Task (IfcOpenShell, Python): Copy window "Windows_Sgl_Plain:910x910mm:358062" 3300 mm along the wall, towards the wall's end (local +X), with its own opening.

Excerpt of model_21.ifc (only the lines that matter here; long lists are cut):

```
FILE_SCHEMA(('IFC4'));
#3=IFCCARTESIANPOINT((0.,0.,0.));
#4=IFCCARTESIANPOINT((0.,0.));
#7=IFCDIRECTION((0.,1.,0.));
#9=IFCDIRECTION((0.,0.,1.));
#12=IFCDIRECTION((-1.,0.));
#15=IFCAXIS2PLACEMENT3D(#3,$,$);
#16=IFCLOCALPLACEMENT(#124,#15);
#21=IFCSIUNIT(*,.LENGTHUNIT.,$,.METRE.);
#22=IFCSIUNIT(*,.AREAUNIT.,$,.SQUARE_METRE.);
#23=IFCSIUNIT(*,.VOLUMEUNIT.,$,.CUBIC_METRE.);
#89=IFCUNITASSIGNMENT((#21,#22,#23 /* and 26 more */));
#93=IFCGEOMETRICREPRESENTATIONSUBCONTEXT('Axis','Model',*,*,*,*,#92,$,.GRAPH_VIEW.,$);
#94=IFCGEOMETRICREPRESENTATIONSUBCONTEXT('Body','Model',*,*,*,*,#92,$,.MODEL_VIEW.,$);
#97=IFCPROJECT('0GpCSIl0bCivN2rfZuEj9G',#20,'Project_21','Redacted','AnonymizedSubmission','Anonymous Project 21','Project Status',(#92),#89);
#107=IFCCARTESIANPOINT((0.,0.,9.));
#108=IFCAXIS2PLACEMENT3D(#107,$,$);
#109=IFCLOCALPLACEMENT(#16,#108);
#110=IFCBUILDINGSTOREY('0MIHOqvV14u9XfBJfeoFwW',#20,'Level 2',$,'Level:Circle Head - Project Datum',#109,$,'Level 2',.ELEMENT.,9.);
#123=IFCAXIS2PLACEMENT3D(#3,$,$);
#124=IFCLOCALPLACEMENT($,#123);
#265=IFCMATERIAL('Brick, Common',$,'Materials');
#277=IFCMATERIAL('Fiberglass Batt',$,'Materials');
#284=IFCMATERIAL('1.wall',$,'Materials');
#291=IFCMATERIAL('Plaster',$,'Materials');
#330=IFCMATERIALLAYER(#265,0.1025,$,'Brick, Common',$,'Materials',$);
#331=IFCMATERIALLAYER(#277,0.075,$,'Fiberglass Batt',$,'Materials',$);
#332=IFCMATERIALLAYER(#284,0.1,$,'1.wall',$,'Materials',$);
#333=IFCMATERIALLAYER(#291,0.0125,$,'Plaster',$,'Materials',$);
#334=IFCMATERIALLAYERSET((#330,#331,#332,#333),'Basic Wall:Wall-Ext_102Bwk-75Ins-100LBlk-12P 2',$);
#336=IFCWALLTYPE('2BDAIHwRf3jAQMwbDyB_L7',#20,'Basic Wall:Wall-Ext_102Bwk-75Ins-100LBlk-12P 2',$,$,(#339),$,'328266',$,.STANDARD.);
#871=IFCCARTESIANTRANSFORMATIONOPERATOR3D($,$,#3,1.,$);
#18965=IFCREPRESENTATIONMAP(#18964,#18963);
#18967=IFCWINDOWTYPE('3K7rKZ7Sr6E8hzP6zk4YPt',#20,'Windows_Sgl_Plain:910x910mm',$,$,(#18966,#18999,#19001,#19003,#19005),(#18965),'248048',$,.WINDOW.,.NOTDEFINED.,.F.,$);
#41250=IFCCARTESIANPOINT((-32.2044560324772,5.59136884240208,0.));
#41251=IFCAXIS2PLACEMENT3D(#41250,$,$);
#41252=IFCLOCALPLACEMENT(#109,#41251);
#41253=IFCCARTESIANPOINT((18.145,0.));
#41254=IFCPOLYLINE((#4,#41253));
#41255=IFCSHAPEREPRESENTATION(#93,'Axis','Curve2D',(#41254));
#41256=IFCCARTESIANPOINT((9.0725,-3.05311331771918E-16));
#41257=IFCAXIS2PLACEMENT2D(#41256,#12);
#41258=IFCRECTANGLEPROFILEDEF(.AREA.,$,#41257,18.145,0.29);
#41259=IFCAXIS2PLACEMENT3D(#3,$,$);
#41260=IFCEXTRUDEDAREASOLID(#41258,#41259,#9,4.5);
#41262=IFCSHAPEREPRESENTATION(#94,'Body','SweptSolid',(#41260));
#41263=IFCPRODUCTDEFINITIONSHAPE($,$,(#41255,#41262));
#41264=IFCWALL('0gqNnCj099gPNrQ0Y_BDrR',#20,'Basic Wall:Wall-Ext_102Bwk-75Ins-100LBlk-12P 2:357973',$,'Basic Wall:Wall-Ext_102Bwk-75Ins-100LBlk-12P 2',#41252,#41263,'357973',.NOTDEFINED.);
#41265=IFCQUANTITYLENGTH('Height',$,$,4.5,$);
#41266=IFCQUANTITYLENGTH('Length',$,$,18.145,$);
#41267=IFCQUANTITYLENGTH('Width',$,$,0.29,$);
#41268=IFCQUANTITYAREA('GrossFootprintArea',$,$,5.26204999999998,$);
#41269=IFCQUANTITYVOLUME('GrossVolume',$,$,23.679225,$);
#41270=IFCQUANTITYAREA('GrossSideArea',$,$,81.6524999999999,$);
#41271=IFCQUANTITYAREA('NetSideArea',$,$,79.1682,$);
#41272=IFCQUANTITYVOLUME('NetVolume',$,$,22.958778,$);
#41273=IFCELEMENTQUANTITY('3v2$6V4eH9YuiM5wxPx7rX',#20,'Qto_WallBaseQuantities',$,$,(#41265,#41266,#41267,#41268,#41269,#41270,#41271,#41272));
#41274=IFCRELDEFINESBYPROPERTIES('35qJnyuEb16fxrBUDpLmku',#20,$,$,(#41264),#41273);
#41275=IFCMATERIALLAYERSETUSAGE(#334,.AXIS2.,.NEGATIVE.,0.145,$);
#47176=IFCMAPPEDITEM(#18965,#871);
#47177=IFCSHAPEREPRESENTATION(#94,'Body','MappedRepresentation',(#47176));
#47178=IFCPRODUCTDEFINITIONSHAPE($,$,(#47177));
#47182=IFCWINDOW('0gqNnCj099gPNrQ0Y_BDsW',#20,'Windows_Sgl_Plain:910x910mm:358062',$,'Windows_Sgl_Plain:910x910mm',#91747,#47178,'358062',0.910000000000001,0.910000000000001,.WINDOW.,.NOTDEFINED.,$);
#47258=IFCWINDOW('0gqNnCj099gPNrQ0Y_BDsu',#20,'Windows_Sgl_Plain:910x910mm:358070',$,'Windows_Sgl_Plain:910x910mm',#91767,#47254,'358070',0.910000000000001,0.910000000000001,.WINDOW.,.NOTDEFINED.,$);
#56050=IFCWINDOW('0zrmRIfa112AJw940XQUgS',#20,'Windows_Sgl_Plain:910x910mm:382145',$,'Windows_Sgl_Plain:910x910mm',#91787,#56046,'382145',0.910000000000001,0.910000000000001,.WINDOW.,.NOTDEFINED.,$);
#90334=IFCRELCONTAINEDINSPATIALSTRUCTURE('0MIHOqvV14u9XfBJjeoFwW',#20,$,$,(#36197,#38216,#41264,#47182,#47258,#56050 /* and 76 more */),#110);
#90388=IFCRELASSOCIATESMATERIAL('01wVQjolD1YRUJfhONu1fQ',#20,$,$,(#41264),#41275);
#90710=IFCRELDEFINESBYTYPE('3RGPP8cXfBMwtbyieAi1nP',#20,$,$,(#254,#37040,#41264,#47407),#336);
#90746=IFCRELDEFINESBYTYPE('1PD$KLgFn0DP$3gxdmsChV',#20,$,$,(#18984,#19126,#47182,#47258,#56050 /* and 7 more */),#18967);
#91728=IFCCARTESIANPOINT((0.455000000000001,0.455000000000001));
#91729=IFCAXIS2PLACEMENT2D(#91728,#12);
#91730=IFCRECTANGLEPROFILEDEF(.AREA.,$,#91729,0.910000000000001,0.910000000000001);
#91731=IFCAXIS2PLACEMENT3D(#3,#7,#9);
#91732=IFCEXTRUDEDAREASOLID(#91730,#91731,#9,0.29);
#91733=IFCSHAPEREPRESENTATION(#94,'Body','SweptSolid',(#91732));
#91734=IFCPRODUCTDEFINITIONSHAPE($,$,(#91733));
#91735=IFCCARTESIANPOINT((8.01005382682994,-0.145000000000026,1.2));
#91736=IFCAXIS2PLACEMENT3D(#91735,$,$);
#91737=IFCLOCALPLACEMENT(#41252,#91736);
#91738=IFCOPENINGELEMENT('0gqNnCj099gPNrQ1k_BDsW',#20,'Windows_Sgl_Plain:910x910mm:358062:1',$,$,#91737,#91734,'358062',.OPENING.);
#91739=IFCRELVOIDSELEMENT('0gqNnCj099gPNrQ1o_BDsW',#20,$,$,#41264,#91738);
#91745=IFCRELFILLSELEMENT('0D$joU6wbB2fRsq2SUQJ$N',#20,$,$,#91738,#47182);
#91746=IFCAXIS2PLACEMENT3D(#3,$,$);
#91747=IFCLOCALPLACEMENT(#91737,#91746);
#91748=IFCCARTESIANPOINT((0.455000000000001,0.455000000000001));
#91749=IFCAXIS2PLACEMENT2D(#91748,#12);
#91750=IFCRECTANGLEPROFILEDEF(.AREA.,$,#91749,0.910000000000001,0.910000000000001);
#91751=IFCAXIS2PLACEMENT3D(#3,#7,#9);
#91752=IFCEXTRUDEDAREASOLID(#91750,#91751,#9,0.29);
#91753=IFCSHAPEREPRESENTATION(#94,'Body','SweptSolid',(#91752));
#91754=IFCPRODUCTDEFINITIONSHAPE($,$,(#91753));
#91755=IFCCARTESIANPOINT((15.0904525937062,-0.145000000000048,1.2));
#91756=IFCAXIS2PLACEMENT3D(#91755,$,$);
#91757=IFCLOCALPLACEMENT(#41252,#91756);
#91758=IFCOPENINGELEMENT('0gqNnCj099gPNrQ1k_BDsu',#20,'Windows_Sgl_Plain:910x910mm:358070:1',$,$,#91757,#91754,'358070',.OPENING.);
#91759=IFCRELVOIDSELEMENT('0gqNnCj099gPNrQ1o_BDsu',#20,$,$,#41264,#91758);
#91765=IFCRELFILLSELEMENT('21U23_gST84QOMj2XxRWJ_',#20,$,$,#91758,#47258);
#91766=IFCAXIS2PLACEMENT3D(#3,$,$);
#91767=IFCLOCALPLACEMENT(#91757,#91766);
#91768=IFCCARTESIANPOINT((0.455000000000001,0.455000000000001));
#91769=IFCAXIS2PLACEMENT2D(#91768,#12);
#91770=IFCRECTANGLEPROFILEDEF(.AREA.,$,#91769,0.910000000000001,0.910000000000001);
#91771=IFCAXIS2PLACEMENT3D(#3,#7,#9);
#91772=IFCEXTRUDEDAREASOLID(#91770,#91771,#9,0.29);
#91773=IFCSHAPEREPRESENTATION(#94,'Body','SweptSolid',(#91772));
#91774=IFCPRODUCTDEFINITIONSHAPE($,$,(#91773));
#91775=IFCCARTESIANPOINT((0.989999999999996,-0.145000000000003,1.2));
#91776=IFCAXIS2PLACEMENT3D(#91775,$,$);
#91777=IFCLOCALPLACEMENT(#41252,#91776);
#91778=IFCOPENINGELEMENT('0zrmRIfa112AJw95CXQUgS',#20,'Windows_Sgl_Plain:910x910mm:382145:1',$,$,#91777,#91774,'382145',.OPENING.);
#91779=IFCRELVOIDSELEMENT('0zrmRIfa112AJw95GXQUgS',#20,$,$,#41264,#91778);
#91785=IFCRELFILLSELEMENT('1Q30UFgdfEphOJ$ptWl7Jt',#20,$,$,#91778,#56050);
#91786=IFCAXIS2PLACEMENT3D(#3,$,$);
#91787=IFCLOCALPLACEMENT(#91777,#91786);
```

```python
import ifcopenshell
import ifcopenshell.api.feature
import ifcopenshell.api.geometry
import ifcopenshell.api.pset
import ifcopenshell.api.root
import ifcopenshell.geom
import ifcopenshell.util.element
import ifcopenshell.util.placement
import ifcopenshell.util.shape
import ifcopenshell.util.unit

model = ifcopenshell.open("model_21.ifc")
unit_scale = ifcopenshell.util.unit.calculate_unit_scale(model)
area_scale = ifcopenshell.util.unit.calculate_unit_scale(model, "AREAUNIT")
volume_scale = ifcopenshell.util.unit.calculate_unit_scale(model, "VOLUMEUNIT")
settings = ifcopenshell.geom.settings()


def volume(element):
    """Net volume in cubic metres, openings subtracted."""
    shape = ifcopenshell.geom.create_shape(settings, element)
    return ifcopenshell.util.shape.get_volume(shape.geometry)


def reuse_history(source, copy):
    """copy_class also copies each property set's owner history, people and application; keep the originals."""
    for rel in copy.IsDefinedBy:
        if rel.is_a("IfcRelDefinesByProperties") and (history := rel.RelatingPropertyDefinition.OwnerHistory):
            rel.RelatingPropertyDefinition.OwnerHistory = source.OwnerHistory
            ifcopenshell.util.element.remove_deep2(model, history)


window = model.by_id(47182)
opening = window.FillsVoids[0].RelatingOpeningElement
wall = opening.VoidsElements[0].RelatingBuildingElement
before = volume(wall)
shift = ifcopenshell.util.placement.get_local_placement(wall.ObjectPlacement)[:3, 0] * 3.3 / unit_scale

# copy_class copies the void relationship, type, container and properties, but no geometry.
new_opening = ifcopenshell.api.root.copy_class(model, product=opening)
new_opening.Representation = ifcopenshell.util.element.copy_deep(
    model, opening.Representation, exclude=["IfcGeometricRepresentationContext", "IfcRepresentationMap"]
)
new_opening.Name = "Windows_Sgl_Plain:910x910mm"
new_opening.Tag = None
reuse_history(opening, new_opening)
new_window = ifcopenshell.api.root.copy_class(model, product=window)
new_window.Representation = ifcopenshell.util.element.copy_deep(
    model, window.Representation, exclude=["IfcGeometricRepresentationContext", "IfcRepresentationMap"]
)
new_window.Name = "Windows_Sgl_Plain:910x910mm"
new_window.Tag = None
reuse_history(window, new_window)
ifcopenshell.api.feature.add_filling(model, opening=new_opening, element=new_window)

for old, new in ((opening, new_opening), (window, new_window)):
    matrix = ifcopenshell.util.placement.get_local_placement(old.ObjectPlacement)
    matrix[:3, 3] += shift
    ifcopenshell.api.geometry.edit_object_placement(model, product=new, matrix=matrix, is_si=False)

after = volume(wall)
thickness = 0.29  # wall thickness in metres

# Update the wall's stored quantities.
qto = model.by_id(ifcopenshell.util.element.get_pset(wall, "Qto_WallBaseQuantities", should_inherit=False)["id"])
ifcopenshell.api.pset.edit_qto(model, qto=qto, properties={
    "NetSideArea": after / thickness / area_scale,
    "NetVolume": after / volume_scale,
})

print(f"wall volume {before:.3f} -> {after:.3f} m3")

model.write("model_21_updated.ifc")
```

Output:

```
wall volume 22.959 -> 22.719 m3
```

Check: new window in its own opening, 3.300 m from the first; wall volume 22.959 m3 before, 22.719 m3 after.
